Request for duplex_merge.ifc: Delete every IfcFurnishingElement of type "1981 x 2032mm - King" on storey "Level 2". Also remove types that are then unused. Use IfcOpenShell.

First a look at what the model holds.

```python
import ifcopenshell
import ifcopenshell.util.element

model = ifcopenshell.open("duplex_merge.ifc")
print(model.schema)
storey = next(s for s in model.by_type("IfcBuildingStorey") if s.Name == "Level 2")
furniture = [e for e in ifcopenshell.util.element.get_decomposition(storey) if e.is_a("IfcFurnishingElement")]
seen = {}
for e in furniture:
    element_type = ifcopenshell.util.element.get_type(e)
    name = element_type.Name if element_type not in (None, e) else None
    seen[name] = seen.get(name, 0) + 1
for name, count in sorted(seen.items(), key=str):
    print(count, "x", name)
```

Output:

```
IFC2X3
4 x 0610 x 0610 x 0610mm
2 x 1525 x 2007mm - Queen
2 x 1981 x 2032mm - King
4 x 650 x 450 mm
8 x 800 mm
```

```python
import ifcopenshell
import ifcopenshell.api.root
import ifcopenshell.util.element

model = ifcopenshell.open("duplex_merge.ifc")

storey = next(s for s in model.by_type("IfcBuildingStorey") if s.Name == "Level 2")
furniture = [e for e in ifcopenshell.util.element.get_decomposition(storey) if e.is_a("IfcFurnishingElement")]
targets = [e for e in furniture if (t := ifcopenshell.util.element.get_type(e)) not in (None, e) and t.Name == "1981 x 2032mm - King"]
types = {ifcopenshell.util.element.get_type(e) for e in targets} - {None, *targets}

for e in targets:
    ifcopenshell.api.root.remove_product(model, product=e)
print(len(targets), "removed")

unused = [t for t in types if not ifcopenshell.util.element.get_types(t)]
for t in unused:
    ifcopenshell.api.root.remove_product(model, product=t)
print(len(unused), "unused types removed")

model.write("duplex_merge_rev.ifc")
```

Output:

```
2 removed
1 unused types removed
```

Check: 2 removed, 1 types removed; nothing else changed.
